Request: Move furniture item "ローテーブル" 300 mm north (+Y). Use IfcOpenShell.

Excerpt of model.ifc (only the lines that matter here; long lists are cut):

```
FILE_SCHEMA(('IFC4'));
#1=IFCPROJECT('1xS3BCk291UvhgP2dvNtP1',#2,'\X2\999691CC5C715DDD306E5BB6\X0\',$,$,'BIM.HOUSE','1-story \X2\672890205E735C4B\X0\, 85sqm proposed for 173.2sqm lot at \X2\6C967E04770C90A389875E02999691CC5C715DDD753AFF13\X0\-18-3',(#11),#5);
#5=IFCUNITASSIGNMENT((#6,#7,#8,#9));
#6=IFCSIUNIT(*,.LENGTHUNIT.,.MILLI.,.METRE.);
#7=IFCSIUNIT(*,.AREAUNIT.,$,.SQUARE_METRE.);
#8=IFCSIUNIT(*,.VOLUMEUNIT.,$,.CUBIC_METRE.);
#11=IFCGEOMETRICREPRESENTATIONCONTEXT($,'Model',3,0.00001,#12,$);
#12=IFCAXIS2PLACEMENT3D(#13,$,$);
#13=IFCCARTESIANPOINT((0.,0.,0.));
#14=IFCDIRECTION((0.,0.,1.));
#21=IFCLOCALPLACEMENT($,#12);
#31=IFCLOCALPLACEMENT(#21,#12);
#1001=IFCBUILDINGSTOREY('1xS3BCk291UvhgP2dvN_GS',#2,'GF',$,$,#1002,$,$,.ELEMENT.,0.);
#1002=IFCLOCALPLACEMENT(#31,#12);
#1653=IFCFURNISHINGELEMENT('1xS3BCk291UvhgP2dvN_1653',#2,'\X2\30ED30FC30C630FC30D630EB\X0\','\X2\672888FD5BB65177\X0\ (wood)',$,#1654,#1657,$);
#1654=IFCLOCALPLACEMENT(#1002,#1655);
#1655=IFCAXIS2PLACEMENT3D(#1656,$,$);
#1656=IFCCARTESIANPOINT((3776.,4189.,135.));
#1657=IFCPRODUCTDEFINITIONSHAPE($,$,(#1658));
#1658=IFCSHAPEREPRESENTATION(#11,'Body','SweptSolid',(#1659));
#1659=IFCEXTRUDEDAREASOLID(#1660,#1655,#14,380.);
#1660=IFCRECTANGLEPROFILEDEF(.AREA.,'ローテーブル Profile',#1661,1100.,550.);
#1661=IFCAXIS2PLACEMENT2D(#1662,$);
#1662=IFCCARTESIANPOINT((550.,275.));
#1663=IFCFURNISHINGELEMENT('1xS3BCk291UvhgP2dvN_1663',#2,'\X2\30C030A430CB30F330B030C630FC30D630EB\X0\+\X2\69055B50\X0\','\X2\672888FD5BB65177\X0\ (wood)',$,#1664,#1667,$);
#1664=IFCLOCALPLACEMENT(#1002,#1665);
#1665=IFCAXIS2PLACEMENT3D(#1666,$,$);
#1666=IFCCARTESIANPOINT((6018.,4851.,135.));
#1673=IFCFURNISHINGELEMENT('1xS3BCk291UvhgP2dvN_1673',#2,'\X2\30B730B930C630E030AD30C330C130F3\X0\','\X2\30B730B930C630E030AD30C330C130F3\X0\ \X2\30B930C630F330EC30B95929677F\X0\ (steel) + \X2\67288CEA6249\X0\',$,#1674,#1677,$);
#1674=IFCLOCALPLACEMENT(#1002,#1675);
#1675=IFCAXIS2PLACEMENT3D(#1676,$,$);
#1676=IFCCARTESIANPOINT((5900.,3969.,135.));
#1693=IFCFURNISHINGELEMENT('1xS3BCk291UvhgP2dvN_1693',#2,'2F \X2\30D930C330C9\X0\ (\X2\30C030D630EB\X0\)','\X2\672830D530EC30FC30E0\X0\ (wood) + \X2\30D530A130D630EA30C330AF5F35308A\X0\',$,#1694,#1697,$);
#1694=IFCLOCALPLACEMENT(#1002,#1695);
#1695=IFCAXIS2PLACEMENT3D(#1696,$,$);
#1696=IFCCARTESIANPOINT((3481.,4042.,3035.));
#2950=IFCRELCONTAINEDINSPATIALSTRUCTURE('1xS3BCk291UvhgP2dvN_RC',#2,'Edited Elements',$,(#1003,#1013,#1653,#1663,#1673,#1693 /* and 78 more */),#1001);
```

```python
import ifcopenshell
import ifcopenshell.api.geometry
import ifcopenshell.util.placement

model = ifcopenshell.open("model.ifc")

item = model.by_id(1653)
matrix = ifcopenshell.util.placement.get_local_placement(item.ObjectPlacement)
matrix[1, 3] += 300.0
ifcopenshell.api.geometry.edit_object_placement(model, product=item, matrix=matrix, is_si=False)

print(ifcopenshell.util.placement.get_local_placement(item.ObjectPlacement).round(3) + 0.0)

model.write("model_v2.ifc")
```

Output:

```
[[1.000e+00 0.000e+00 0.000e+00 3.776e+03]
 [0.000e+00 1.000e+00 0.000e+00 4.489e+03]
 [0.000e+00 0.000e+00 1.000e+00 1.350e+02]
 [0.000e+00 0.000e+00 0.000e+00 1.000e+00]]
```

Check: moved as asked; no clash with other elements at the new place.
